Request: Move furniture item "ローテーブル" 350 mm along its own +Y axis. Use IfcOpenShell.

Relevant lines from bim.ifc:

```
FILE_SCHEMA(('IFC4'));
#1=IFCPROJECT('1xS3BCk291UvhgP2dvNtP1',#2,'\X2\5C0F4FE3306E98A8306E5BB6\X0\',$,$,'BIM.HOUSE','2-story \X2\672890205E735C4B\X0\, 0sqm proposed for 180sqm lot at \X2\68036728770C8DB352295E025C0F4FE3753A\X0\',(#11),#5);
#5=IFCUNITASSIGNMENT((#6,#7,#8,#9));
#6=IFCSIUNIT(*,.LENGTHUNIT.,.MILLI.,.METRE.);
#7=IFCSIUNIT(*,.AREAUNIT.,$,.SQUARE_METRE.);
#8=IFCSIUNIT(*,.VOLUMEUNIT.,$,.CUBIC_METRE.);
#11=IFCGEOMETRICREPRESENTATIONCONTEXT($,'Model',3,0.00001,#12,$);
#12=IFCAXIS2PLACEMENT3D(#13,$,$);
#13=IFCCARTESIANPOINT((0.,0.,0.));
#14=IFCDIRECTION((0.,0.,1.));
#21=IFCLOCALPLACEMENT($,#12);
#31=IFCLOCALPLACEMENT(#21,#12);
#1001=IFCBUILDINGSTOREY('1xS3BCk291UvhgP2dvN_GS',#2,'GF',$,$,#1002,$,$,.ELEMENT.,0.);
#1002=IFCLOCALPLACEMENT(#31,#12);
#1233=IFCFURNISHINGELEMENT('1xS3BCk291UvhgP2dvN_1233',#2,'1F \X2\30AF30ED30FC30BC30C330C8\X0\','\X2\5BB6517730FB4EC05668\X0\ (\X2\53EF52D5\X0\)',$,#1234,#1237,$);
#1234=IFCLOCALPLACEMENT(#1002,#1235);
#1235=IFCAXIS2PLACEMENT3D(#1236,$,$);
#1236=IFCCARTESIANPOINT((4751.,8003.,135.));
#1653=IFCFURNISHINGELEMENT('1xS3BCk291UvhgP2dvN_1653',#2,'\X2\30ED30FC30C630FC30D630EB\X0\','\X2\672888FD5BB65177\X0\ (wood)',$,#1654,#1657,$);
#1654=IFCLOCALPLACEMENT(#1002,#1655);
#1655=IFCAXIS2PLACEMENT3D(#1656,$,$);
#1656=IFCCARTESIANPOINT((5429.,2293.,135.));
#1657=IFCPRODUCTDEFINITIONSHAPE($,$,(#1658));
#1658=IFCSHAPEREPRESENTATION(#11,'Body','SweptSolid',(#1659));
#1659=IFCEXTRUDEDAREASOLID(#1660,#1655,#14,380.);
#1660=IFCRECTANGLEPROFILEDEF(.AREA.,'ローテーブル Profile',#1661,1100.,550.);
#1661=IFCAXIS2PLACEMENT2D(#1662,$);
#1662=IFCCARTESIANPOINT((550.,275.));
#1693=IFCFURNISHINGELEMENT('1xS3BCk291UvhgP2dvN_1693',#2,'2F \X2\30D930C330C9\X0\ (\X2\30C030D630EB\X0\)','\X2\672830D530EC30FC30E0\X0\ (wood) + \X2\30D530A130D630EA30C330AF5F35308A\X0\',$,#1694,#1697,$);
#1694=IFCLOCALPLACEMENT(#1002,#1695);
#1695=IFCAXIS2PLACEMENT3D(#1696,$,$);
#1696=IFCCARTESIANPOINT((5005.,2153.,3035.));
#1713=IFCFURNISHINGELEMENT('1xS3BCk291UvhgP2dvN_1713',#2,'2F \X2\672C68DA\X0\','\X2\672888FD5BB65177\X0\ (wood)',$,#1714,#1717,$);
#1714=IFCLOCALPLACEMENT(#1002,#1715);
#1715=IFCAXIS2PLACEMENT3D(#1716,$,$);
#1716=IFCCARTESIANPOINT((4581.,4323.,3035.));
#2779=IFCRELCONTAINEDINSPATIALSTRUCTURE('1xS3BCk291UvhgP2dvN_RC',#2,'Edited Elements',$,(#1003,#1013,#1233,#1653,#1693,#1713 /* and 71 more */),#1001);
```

```python
import ifcopenshell
import ifcopenshell.api.geometry
import ifcopenshell.util.placement

model = ifcopenshell.open("bim.ifc")

item = model.by_id(1653)
matrix = ifcopenshell.util.placement.get_local_placement(item.ObjectPlacement)
matrix[:3, 3] += matrix[:3, 1] * 350.0
ifcopenshell.api.geometry.edit_object_placement(model, product=item, matrix=matrix, is_si=False)

print(ifcopenshell.util.placement.get_local_placement(item.ObjectPlacement).round(3) + 0.0)

model.write("bim-out.ifc")
```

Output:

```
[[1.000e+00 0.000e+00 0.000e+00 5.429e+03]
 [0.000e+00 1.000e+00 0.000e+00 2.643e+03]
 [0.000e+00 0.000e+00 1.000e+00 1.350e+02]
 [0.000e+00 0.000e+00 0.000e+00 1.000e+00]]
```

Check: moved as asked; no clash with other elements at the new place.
